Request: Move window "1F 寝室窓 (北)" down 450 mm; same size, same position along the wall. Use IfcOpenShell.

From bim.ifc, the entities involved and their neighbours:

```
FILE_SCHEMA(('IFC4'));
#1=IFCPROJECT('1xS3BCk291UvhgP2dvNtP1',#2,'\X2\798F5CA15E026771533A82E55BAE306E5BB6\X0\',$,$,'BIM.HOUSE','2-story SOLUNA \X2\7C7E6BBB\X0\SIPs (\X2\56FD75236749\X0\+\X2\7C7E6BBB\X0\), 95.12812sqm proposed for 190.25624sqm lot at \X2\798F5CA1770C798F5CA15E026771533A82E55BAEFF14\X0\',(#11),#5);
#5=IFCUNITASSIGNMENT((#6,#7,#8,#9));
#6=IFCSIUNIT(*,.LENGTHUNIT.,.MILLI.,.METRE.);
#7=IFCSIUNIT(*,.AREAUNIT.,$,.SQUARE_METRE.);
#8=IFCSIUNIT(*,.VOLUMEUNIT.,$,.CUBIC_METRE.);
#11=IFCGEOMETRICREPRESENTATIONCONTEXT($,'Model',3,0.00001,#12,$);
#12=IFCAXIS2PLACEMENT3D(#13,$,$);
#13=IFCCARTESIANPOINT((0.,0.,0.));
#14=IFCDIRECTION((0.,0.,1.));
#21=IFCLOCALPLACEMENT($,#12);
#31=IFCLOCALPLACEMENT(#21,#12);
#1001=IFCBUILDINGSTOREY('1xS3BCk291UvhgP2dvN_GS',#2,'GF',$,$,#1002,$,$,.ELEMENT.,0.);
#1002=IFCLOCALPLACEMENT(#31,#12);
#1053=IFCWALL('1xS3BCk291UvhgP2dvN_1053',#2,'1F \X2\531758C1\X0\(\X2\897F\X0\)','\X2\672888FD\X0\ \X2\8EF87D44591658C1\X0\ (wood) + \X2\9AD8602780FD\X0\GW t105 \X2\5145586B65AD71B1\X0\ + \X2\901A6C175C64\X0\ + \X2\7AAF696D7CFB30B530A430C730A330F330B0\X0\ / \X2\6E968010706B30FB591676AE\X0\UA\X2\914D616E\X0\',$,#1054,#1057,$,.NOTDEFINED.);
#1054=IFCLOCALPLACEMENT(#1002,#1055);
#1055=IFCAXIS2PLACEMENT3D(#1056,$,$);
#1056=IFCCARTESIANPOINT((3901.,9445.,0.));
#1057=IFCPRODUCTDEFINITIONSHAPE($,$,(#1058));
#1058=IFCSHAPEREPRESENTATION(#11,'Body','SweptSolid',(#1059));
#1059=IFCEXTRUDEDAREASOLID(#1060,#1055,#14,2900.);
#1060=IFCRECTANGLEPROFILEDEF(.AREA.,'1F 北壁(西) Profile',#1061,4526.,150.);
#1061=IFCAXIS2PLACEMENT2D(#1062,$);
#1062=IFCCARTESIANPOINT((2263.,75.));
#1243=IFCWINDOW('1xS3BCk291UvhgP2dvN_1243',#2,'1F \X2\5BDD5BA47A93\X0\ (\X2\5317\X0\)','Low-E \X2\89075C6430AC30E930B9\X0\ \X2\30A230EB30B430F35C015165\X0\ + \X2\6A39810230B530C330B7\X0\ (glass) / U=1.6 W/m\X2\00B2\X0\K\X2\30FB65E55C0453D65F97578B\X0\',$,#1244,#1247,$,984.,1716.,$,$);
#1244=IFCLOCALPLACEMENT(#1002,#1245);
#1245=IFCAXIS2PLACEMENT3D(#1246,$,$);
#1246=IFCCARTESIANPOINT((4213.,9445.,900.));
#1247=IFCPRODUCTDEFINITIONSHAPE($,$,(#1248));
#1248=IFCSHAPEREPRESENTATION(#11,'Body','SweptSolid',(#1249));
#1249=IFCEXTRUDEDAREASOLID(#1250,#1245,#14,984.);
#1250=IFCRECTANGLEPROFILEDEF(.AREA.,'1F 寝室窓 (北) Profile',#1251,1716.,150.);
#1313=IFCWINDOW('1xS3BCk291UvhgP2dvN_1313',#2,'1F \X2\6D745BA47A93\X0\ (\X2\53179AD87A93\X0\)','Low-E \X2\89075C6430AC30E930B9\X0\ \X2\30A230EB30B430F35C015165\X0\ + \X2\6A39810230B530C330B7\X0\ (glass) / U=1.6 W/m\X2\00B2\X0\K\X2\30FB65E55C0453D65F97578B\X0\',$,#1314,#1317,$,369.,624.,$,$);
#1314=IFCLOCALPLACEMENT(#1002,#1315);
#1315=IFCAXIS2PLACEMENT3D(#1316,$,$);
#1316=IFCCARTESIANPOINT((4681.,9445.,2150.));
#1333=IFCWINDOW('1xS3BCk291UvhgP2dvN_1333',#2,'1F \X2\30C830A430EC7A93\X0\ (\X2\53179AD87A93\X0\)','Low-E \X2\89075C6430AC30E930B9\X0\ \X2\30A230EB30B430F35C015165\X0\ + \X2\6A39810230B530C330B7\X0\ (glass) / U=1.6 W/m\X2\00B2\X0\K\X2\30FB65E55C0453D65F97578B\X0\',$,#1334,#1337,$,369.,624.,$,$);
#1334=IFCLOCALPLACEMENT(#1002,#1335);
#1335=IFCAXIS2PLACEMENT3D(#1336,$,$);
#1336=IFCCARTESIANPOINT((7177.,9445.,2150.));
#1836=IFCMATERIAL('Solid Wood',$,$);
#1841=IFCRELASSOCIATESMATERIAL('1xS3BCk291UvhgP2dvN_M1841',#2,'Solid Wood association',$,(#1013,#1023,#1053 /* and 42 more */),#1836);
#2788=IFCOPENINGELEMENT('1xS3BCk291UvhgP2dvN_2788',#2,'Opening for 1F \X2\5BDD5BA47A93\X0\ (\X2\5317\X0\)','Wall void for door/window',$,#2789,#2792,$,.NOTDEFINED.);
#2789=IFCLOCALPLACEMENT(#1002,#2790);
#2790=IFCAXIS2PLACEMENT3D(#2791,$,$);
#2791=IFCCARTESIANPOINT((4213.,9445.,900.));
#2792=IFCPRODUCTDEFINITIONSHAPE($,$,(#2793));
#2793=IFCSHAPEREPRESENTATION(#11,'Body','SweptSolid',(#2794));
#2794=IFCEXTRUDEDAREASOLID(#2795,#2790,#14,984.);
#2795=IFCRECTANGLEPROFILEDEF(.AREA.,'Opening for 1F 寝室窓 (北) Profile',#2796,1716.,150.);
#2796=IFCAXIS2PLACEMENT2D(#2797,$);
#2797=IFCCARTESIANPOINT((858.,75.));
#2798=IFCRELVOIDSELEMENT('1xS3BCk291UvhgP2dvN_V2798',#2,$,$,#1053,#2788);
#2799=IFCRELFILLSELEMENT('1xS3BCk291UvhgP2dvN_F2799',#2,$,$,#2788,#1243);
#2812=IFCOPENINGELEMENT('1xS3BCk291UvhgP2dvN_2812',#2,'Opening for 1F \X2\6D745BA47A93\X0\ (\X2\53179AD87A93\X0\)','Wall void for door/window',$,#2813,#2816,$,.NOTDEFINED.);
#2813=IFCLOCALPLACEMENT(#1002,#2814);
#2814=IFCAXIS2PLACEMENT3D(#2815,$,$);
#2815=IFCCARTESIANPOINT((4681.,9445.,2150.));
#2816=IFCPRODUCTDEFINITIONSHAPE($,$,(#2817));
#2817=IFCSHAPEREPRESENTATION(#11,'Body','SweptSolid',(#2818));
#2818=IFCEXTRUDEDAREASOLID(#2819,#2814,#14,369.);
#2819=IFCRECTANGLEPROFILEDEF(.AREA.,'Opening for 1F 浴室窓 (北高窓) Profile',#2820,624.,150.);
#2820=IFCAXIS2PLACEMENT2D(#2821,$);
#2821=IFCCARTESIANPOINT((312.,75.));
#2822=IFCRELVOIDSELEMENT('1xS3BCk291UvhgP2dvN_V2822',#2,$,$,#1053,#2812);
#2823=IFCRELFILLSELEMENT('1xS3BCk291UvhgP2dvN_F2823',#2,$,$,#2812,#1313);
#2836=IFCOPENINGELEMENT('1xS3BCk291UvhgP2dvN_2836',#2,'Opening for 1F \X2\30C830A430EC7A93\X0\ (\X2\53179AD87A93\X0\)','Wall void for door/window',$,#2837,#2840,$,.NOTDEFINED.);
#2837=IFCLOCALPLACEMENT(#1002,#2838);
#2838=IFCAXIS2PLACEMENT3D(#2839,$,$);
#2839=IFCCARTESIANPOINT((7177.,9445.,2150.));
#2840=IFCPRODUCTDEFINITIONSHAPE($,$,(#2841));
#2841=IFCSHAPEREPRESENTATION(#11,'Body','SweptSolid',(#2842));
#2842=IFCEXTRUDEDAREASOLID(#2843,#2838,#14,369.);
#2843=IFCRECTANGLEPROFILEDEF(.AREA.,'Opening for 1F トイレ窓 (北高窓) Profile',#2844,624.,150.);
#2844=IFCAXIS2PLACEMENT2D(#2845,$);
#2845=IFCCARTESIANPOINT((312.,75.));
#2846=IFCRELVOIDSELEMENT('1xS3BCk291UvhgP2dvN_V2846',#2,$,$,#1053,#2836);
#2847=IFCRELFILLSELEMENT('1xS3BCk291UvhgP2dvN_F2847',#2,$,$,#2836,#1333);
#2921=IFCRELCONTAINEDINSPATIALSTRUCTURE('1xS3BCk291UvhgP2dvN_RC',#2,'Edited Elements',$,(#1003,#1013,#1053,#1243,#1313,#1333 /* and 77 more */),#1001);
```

```python
import numpy as np
import ifcopenshell
import ifcopenshell.api.geometry
import ifcopenshell.util.placement
import ifcopenshell.util.unit

model = ifcopenshell.open("bim.ifc")
unit_scale = ifcopenshell.util.unit.calculate_unit_scale(model)

window = model.by_guid("1xS3BCk291UvhgP2dvN_1243")
opening = window.FillsVoids[0].RelatingOpeningElement
dz = -0.45 / unit_scale

shift = np.array([0.0, 0.0, dz])
# The window is not placed relative to its opening, so move both.
for product in (opening, window):
    matrix = ifcopenshell.util.placement.get_local_placement(product.ObjectPlacement)
    matrix[:3, 3] += shift
    ifcopenshell.api.geometry.edit_object_placement(model, product=product, matrix=matrix, is_si=False)

print(f"moved by {dz * unit_scale:+.3f} m")

model.write("bim_updated.ifc")
```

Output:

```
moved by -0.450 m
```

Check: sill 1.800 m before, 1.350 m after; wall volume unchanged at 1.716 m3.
